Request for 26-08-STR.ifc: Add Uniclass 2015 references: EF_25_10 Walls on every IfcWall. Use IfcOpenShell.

First a look at what the model holds.

```python
import ifcopenshell

model = ifcopenshell.open("26-08-STR.ifc")
print(model.schema)
print("classifications:", [c.Name for c in model.by_type("IfcClassification")])
for ifc_class in ("IfcDoor", "IfcRoof", "IfcStair", "IfcWall", "IfcWindow"):
    print(ifc_class, len(model.by_type(ifc_class)))
```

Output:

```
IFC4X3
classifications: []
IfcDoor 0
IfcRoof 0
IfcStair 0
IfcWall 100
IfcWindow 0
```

```python
import ifcopenshell
import ifcopenshell.api.classification

model = ifcopenshell.open("26-08-STR.ifc")

system = ifcopenshell.api.classification.add_classification(model, classification="Uniclass 2015")

codes = {
    "IfcWall": ("EF_25_10", "Walls"),
}
for ifc_class, (code, name) in codes.items():
    products = model.by_type(ifc_class)
    ifcopenshell.api.classification.add_reference(
        model, products=products, classification=system, identification=code, name=name
    )
    print(code, len(products))

model.write("26-08-STR_v2.ifc")
```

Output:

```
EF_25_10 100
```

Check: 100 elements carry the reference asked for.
